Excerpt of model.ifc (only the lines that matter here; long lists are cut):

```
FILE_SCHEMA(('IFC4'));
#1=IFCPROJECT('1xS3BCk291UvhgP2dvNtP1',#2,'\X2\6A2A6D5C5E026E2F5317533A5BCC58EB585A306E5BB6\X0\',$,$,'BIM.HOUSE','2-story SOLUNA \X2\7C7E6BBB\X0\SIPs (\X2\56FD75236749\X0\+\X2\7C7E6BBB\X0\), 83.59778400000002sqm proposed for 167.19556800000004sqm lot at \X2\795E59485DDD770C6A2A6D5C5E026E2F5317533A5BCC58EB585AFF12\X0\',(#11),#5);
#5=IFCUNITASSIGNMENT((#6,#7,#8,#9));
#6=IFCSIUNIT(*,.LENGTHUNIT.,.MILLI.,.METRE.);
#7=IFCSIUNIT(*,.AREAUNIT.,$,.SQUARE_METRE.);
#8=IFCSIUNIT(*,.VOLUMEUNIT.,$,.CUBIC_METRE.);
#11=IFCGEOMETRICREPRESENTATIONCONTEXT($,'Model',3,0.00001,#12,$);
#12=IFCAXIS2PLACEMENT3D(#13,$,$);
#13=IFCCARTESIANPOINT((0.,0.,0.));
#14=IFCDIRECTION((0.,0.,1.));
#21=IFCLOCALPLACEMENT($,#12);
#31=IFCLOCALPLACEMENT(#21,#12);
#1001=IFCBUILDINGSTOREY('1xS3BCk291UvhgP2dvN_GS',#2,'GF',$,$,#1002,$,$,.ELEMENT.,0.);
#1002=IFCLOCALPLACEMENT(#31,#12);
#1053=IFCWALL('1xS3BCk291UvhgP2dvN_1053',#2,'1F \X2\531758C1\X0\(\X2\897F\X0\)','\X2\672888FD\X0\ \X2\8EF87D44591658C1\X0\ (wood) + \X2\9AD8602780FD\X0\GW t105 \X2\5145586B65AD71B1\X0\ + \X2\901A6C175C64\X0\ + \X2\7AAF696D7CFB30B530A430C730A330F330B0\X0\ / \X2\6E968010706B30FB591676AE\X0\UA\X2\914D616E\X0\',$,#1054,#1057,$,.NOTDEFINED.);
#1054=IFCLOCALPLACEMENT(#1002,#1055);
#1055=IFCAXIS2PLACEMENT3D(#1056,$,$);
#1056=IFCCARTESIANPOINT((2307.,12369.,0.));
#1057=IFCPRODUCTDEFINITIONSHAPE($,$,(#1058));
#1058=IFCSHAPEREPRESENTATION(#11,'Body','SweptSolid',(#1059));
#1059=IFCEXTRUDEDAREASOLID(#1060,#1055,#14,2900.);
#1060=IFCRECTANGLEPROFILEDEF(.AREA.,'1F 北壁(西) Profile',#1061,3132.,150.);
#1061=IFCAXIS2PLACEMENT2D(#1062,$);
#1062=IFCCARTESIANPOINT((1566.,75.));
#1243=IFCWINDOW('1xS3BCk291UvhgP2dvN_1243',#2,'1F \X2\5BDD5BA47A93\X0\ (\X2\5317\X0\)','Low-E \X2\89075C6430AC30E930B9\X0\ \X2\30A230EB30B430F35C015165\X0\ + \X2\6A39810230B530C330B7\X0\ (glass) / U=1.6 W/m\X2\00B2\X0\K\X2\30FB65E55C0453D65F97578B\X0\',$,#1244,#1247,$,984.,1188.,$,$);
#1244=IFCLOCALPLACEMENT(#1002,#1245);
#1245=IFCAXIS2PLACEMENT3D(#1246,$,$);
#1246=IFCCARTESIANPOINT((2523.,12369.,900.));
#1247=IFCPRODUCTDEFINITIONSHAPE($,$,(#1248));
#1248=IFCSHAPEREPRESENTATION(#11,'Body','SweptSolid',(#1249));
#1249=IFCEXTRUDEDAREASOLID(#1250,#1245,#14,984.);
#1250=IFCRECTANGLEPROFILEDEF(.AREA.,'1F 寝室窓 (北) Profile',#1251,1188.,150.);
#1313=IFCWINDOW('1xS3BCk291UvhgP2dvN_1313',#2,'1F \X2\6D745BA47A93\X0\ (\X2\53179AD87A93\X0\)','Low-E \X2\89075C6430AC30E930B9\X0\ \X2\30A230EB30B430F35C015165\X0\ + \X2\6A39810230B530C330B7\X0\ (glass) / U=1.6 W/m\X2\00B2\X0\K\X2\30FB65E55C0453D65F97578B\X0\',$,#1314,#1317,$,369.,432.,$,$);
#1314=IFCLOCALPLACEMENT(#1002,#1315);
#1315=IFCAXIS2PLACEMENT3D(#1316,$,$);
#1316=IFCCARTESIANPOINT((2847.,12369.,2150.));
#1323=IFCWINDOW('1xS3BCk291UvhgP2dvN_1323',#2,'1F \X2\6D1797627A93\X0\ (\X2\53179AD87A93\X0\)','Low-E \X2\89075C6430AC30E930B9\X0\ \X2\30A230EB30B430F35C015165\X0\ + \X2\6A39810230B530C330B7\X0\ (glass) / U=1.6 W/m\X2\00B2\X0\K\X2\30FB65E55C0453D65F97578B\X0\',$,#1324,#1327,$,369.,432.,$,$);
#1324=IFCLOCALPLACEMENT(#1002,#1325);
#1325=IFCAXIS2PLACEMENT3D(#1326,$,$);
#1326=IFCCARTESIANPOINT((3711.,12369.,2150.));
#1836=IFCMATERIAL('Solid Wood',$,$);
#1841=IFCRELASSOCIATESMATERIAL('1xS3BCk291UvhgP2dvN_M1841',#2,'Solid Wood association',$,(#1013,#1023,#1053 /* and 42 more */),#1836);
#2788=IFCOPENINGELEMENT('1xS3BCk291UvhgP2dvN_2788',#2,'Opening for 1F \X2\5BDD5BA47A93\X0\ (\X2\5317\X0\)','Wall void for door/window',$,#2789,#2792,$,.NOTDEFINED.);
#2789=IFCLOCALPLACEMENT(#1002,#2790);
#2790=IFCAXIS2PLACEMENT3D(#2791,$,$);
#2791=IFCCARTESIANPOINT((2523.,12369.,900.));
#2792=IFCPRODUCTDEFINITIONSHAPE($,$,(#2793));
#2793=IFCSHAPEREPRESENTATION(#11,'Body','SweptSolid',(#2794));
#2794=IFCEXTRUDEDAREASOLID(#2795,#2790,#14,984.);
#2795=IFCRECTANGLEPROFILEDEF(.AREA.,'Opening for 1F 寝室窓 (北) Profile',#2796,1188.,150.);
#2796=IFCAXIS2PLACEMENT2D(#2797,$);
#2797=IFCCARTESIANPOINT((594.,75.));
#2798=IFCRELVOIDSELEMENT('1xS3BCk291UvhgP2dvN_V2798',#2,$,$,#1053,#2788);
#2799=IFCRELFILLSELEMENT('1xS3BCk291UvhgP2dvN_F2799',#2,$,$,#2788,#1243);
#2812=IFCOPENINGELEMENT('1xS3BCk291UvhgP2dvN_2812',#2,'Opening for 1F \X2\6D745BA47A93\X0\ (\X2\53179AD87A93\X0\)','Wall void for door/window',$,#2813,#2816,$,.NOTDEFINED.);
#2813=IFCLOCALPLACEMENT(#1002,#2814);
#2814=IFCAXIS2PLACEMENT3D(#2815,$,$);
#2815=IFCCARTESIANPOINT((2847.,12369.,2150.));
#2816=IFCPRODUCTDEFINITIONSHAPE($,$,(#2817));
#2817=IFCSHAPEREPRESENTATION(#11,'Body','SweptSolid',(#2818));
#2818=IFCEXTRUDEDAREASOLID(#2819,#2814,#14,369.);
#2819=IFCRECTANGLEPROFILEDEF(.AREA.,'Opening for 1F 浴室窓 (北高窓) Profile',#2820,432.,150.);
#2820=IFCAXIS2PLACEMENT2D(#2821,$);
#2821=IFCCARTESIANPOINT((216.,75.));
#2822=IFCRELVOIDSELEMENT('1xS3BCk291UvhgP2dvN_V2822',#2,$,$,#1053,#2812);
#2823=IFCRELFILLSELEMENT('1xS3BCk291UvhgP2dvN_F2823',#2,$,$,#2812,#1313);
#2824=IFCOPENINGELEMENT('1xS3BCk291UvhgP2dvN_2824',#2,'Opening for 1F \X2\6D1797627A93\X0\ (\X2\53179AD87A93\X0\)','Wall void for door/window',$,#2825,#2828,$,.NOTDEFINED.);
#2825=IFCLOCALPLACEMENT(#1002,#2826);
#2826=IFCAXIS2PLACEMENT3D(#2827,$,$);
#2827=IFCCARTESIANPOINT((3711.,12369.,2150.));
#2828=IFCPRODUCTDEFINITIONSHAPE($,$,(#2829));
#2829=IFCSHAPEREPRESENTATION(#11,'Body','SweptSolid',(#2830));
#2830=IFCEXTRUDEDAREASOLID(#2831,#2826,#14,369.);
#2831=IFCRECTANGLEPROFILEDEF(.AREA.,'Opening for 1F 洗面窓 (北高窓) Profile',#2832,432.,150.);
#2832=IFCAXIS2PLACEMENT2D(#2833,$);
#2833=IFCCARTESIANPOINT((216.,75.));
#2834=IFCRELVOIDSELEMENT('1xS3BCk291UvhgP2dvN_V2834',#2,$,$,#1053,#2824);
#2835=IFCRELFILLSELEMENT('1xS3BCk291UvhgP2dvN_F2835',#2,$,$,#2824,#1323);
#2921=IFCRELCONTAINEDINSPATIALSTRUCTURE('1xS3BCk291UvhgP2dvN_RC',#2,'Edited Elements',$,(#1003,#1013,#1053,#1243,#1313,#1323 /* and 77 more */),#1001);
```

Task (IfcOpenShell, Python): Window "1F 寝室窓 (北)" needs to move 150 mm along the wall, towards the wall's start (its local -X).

```python
import ifcopenshell
import ifcopenshell.api.geometry
import ifcopenshell.util.placement

model = ifcopenshell.open("model.ifc")

window = model.by_guid("1xS3BCk291UvhgP2dvN_1243")
opening = window.FillsVoids[0].RelatingOpeningElement
wall = opening.VoidsElements[0].RelatingBuildingElement

wall_matrix = ifcopenshell.util.placement.get_local_placement(wall.ObjectPlacement)
shift = wall_matrix[:3, 0] * -150.0
before = ifcopenshell.util.placement.get_local_placement(window.ObjectPlacement)[:3, 3].copy()

# The window is not placed relative to its opening, so move both.
for product in (opening, window):
    matrix = ifcopenshell.util.placement.get_local_placement(product.ObjectPlacement)
    matrix[:3, 3] += shift
    ifcopenshell.api.geometry.edit_object_placement(model, product=product, matrix=matrix, is_si=False)

after = ifcopenshell.util.placement.get_local_placement(window.ObjectPlacement)[:3, 3]
print("window moved by", (after - before).round(3) + 0.0)

model.write("model-out.ifc")
```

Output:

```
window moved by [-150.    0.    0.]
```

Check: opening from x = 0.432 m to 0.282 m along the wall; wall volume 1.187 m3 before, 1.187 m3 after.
